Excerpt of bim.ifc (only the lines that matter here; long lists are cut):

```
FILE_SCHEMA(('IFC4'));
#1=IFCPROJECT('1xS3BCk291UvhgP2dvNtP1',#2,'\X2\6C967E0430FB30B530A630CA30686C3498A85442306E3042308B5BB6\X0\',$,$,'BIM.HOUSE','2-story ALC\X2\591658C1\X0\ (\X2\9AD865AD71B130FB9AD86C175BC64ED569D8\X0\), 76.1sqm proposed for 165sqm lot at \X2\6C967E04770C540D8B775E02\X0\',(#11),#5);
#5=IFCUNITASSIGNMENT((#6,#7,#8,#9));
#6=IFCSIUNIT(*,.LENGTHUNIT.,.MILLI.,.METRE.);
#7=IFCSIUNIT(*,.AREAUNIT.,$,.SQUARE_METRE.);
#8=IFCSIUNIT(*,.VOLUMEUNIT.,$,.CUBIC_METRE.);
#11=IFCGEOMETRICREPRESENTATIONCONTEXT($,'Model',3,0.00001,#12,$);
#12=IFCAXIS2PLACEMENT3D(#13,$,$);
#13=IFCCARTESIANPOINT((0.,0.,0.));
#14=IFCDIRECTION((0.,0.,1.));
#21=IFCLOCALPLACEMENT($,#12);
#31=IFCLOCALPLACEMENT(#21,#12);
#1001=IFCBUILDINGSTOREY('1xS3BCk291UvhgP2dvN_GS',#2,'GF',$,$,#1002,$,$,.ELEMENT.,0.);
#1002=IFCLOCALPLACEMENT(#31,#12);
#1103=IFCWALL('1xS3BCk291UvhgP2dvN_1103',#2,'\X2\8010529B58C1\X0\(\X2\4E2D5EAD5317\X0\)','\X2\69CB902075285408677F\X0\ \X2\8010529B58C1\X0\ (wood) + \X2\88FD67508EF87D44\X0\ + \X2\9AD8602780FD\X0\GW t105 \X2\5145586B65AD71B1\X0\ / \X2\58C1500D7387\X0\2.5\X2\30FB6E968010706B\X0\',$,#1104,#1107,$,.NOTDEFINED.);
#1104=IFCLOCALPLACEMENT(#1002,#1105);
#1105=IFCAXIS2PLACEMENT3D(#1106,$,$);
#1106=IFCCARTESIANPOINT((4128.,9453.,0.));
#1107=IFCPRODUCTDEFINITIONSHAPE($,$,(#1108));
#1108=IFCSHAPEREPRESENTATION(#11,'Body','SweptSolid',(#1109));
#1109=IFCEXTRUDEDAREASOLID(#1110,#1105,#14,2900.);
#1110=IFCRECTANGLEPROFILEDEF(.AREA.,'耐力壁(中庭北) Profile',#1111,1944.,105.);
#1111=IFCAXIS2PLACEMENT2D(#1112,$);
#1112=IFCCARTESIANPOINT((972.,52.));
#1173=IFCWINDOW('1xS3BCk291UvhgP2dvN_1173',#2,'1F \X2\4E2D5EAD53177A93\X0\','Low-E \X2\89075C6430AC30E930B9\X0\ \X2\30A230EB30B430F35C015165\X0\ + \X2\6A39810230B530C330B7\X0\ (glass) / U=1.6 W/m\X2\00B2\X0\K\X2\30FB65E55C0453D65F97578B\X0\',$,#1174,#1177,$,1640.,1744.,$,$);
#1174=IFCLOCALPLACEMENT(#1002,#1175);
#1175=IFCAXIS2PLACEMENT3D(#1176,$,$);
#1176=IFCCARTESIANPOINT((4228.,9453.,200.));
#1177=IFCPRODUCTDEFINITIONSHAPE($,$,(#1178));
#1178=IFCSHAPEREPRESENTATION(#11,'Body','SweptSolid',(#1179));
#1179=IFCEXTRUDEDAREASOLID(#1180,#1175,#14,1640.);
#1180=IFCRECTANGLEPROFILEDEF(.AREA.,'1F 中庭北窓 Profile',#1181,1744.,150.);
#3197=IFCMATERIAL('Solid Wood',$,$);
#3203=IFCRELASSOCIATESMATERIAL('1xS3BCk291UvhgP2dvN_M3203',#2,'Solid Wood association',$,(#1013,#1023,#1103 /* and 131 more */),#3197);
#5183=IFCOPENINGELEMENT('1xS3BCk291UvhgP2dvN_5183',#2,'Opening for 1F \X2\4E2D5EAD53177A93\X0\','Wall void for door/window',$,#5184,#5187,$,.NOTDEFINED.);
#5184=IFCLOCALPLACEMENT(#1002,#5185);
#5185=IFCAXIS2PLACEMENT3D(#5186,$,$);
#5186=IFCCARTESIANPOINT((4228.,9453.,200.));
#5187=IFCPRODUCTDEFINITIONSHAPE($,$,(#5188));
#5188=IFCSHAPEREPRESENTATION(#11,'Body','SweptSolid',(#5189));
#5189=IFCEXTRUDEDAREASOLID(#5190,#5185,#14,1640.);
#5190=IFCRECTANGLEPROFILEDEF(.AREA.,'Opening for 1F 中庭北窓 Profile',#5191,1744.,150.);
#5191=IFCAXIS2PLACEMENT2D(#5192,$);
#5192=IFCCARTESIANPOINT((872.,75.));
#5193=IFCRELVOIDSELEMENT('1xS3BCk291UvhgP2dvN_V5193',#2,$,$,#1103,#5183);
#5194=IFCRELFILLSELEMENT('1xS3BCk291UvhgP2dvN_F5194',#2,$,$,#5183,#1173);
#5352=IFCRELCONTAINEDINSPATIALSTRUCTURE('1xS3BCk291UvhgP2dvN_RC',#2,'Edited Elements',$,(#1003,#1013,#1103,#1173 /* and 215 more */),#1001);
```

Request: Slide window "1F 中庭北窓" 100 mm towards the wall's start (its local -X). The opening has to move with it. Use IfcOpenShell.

```python
import ifcopenshell
import ifcopenshell.api.geometry
import ifcopenshell.util.placement

model = ifcopenshell.open("bim.ifc")

window = model.by_id(1173)
opening = window.FillsVoids[0].RelatingOpeningElement
wall = opening.VoidsElements[0].RelatingBuildingElement

wall_matrix = ifcopenshell.util.placement.get_local_placement(wall.ObjectPlacement)
shift = wall_matrix[:3, 0] * -100.0
before = ifcopenshell.util.placement.get_local_placement(window.ObjectPlacement)[:3, 3].copy()

# The window is not placed relative to its opening, so move both.
for product in (opening, window):
    matrix = ifcopenshell.util.placement.get_local_placement(product.ObjectPlacement)
    matrix[:3, 3] += shift
    ifcopenshell.api.geometry.edit_object_placement(model, product=product, matrix=matrix, is_si=False)

after = ifcopenshell.util.placement.get_local_placement(window.ObjectPlacement)[:3, 3]
print("window moved by", (after - before).round(3) + 0.0)

model.write("bim_edited.ifc")
```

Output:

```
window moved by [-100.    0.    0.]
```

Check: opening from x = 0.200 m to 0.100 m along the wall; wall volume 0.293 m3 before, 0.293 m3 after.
